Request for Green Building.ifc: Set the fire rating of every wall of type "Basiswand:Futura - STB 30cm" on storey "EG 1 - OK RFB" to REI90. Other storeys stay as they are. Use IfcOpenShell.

First a look at what the model holds.

```python
import ifcopenshell
import ifcopenshell.util.element

model = ifcopenshell.open("Green Building.ifc")
print(model.schema)
storey = next(s for s in model.by_type("IfcBuildingStorey") if s.Name == "EG 1 - OK RFB")
walls = [e for e in ifcopenshell.util.element.get_decomposition(storey) if e.is_a("IfcWall")]
seen = {}
for e in walls:
    element_type = ifcopenshell.util.element.get_type(e)
    key = (element_type.Name if element_type != e and element_type else None, ifcopenshell.util.element.get_pset(e, "Pset_WallCommon", "FireRating"))
    seen[key] = seen.get(key, 0) + 1
for (name, value), count in sorted(seen.items(), key=str):
    print(count, "x", name, "|", value)
```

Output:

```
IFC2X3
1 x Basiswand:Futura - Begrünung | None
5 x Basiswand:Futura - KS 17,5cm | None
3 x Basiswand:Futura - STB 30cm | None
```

```python
import ifcopenshell
import ifcopenshell.api.pset
import ifcopenshell.util.element

model = ifcopenshell.open("Green Building.ifc")

storey = next(s for s in model.by_type("IfcBuildingStorey") if s.Name == "EG 1 - OK RFB")
walls = [e for e in ifcopenshell.util.element.get_decomposition(storey) if e.is_a("IfcWall")]

count = 0
for e in walls:
    element_type = ifcopenshell.util.element.get_type(e)
    if element_type in (None, e) or element_type.Name != "Basiswand:Futura - STB 30cm":
        continue
    # add_pset returns the element's existing set when there is one.
    pset = ifcopenshell.api.pset.add_pset(model, product=e, name="Pset_WallCommon")
    ifcopenshell.api.pset.edit_pset(model, pset=pset, properties={"FireRating": "REI90"})
    count += 1

print(count, "walls updated")

model.write("Green Building_rev.ifc")
```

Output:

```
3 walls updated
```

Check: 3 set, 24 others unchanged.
